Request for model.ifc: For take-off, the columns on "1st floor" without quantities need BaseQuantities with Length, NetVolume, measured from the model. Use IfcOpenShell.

First a look at what the model holds.

```python
import ifcopenshell
import ifcopenshell.util.element
import ifcopenshell.util.unit

model = ifcopenshell.open("model.ifc")
print(model.schema)
for unit_type in ("LENGTHUNIT", "AREAUNIT", "VOLUMEUNIT"):
    print(unit_type, ifcopenshell.util.unit.calculate_unit_scale(model, unit_type))
storey = next(s for s in model.by_type("IfcBuildingStorey") if s.Name == "1st floor")
columns = [e for e in ifcopenshell.util.element.get_decomposition(storey) if e.is_a("IfcColumn")]
for e in sorted(columns, key=lambda e: e.id()):
    print(e.id(), e.is_a(), e.Name, list(ifcopenshell.util.element.get_psets(e, qtos_only=True)), sep=" | ")
```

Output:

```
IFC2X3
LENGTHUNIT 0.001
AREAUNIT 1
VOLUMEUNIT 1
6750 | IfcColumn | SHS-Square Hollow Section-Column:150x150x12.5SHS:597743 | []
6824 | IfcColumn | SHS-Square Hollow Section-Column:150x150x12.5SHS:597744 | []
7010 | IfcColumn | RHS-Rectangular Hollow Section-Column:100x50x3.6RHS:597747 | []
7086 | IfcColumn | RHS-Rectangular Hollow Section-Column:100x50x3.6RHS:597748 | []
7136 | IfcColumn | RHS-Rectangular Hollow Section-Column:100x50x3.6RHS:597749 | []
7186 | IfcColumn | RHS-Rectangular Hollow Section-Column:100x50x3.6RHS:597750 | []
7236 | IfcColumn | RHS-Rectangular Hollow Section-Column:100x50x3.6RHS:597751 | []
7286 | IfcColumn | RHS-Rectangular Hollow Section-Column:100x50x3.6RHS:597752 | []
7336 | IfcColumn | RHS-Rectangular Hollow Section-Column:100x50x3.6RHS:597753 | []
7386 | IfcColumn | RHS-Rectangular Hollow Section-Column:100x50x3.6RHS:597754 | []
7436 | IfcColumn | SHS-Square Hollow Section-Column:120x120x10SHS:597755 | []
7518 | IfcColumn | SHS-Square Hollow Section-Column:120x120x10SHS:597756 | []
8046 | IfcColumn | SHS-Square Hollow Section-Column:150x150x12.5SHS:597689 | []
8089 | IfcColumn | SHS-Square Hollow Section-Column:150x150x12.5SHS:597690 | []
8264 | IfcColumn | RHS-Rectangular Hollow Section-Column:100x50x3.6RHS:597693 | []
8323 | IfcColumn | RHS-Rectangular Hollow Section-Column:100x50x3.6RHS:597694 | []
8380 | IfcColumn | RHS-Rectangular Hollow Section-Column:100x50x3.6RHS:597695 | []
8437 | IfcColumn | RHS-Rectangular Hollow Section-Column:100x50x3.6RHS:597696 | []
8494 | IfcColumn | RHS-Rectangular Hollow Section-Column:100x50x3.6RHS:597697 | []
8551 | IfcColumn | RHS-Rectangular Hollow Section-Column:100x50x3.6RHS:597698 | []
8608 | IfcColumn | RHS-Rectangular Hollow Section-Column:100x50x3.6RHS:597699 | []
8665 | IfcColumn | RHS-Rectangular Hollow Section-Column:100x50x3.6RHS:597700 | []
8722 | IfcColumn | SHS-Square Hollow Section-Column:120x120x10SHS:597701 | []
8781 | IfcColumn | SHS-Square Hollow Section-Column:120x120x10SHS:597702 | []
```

```python
import ifcopenshell
import ifcopenshell.api.pset
import ifcopenshell.geom
import ifcopenshell.util.element
import ifcopenshell.util.shape
import ifcopenshell.util.unit

model = ifcopenshell.open("model.ifc")
unit_scale = ifcopenshell.util.unit.calculate_unit_scale(model)
volume_scale = ifcopenshell.util.unit.calculate_unit_scale(model, "VOLUMEUNIT")
settings = ifcopenshell.geom.settings()

storey = next(s for s in model.by_type("IfcBuildingStorey") if s.Name == "1st floor")
columns = [e for e in ifcopenshell.util.element.get_decomposition(storey) if e.is_a("IfcColumn")]

for e in sorted(columns, key=lambda e: e.id()):
    if ifcopenshell.util.element.get_psets(e, qtos_only=True, should_inherit=False):
        continue
    # Geometry comes back in metres, in the element's own axes.
    shape = ifcopenshell.geom.create_shape(settings, e)
    values = {
        "Length": ifcopenshell.util.shape.get_z(shape.geometry) / unit_scale,
        "NetVolume": ifcopenshell.util.shape.get_volume(shape.geometry) / volume_scale,
    }
    qto = ifcopenshell.api.pset.add_qto(model, product=e, name="BaseQuantities")
    ifcopenshell.api.pset.edit_qto(model, qto=qto, properties=values)
    print(e.id(), {k: round(v, 3) for k, v in values.items()})

model.write("model_updated.ifc")
```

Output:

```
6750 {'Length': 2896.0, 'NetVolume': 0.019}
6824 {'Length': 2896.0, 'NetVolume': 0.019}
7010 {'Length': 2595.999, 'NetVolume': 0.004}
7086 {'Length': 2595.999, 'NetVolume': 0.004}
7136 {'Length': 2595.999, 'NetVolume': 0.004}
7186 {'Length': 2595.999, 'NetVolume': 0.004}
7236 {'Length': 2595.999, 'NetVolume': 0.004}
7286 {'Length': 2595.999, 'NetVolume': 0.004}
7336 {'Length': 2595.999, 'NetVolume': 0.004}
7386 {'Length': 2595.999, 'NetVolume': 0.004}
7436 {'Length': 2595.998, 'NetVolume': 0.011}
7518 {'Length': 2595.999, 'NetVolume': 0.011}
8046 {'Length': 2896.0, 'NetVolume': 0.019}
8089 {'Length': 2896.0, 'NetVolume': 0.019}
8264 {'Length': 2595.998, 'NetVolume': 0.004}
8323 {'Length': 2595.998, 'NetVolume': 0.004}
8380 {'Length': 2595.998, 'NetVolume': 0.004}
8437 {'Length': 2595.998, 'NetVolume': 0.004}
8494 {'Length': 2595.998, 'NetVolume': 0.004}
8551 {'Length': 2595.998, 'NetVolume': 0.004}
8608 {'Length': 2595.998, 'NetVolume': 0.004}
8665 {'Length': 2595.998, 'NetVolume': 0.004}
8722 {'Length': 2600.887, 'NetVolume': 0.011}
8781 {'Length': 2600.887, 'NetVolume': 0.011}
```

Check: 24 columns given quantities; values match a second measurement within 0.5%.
